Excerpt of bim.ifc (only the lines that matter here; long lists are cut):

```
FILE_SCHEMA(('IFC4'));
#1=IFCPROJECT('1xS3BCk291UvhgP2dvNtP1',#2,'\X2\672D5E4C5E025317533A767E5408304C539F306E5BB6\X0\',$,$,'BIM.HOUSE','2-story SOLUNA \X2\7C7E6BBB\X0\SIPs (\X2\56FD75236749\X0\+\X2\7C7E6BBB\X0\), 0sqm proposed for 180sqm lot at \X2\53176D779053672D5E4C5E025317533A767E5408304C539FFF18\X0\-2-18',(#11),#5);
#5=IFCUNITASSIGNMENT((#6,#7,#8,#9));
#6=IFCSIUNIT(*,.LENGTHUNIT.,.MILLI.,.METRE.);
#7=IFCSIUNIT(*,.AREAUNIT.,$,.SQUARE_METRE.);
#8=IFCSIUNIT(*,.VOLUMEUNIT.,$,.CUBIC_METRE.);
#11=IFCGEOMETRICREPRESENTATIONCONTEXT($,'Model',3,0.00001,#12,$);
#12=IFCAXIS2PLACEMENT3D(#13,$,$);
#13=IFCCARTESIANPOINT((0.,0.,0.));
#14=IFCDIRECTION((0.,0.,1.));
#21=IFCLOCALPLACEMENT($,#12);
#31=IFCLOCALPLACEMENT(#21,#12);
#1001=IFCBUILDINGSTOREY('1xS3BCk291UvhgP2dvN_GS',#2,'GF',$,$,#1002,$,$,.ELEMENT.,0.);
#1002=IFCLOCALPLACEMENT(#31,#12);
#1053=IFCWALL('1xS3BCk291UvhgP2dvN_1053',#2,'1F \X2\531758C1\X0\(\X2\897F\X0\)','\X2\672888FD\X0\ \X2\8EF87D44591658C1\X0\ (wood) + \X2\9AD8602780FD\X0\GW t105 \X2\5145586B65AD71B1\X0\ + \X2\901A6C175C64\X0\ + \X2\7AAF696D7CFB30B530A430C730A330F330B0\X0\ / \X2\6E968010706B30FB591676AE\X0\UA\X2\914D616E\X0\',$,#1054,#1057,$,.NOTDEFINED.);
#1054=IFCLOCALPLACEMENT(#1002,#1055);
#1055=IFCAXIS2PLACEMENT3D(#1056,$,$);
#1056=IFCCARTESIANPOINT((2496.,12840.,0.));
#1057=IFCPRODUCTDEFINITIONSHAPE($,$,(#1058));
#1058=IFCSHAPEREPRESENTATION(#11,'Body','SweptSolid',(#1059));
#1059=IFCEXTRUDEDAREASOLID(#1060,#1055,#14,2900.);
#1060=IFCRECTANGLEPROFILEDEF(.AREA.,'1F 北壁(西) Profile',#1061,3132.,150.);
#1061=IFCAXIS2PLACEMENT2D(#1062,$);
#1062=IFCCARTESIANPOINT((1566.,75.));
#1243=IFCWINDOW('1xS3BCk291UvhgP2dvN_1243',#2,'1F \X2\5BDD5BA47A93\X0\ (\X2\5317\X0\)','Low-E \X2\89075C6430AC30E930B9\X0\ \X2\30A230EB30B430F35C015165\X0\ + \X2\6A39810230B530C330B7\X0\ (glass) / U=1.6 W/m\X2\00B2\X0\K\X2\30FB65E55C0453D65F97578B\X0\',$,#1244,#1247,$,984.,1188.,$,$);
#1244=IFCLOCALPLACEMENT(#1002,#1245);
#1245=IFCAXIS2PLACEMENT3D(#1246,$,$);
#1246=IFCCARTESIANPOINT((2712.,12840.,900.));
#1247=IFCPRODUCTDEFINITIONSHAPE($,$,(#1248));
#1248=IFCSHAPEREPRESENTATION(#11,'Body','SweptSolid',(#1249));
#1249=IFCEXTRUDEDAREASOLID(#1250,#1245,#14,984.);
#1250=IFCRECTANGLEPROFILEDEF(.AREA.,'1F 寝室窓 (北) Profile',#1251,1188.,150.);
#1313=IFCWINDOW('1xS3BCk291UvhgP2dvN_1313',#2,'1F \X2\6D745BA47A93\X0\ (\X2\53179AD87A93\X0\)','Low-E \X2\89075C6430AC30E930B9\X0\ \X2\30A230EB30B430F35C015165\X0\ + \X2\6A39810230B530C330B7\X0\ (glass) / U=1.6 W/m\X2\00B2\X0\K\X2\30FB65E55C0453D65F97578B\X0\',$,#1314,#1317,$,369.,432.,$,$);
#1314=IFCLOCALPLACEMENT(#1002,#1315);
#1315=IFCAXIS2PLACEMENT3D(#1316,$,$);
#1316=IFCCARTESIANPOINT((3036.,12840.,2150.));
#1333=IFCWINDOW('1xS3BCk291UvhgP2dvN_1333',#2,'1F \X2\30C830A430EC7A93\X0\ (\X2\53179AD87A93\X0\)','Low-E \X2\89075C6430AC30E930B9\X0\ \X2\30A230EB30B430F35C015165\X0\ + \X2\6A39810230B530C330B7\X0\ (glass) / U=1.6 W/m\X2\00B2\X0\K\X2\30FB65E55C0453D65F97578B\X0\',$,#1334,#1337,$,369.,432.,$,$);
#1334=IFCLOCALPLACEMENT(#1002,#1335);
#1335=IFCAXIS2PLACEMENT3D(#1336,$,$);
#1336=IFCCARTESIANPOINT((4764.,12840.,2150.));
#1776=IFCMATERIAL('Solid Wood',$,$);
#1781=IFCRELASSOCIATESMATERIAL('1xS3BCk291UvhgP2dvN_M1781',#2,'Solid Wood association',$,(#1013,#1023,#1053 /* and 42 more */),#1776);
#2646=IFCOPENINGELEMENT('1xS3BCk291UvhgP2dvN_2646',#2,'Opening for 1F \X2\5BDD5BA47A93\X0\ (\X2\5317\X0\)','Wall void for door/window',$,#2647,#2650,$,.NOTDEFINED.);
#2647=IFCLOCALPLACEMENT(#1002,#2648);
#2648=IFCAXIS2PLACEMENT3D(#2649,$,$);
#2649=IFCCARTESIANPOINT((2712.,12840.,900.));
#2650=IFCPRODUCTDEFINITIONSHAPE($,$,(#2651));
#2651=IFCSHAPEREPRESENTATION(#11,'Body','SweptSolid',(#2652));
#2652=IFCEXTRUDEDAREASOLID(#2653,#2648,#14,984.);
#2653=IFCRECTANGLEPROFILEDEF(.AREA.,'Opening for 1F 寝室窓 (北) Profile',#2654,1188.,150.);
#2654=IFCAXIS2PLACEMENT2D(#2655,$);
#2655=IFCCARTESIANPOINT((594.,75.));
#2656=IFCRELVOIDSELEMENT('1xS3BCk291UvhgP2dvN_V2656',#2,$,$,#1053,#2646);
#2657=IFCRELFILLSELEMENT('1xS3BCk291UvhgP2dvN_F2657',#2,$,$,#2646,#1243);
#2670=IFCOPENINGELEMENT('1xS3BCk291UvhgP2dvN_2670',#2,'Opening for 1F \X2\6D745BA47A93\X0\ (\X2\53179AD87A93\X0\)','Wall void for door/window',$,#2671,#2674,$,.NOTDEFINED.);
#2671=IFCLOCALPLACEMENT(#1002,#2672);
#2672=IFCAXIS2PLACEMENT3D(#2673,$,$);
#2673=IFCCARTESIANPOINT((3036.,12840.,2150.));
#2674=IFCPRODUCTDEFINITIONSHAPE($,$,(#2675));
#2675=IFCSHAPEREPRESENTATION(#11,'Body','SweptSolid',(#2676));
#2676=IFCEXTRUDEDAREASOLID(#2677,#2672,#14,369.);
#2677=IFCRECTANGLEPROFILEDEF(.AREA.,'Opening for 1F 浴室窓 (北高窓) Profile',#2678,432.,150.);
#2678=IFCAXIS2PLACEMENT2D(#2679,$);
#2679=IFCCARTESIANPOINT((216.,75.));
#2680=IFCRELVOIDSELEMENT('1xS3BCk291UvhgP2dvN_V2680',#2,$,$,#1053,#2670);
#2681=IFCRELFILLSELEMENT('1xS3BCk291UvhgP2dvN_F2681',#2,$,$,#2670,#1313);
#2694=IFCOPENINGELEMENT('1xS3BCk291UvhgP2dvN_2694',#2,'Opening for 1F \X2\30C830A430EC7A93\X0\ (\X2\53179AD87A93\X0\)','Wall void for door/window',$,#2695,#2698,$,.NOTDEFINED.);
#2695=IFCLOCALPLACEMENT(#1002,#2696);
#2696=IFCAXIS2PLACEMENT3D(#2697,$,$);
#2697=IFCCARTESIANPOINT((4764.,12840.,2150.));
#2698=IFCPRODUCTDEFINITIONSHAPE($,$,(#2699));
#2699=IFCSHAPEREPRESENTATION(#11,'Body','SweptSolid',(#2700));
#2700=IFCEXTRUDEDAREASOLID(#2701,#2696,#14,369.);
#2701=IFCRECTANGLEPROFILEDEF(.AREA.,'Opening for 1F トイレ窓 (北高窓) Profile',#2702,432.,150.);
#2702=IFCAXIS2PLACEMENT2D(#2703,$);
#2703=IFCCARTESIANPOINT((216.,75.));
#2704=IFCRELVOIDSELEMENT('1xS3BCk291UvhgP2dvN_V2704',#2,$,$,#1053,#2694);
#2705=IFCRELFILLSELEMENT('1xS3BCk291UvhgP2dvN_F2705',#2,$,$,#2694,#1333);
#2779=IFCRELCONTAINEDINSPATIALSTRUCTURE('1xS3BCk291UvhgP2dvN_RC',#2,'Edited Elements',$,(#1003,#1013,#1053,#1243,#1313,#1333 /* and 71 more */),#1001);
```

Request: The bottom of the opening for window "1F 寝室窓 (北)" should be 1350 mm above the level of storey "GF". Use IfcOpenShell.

```python
import numpy as np
import ifcopenshell
import ifcopenshell.api.geometry
import ifcopenshell.geom
import ifcopenshell.util.element
import ifcopenshell.util.placement
import ifcopenshell.util.shape
import ifcopenshell.util.unit

model = ifcopenshell.open("bim.ifc")
unit_scale = ifcopenshell.util.unit.calculate_unit_scale(model)

window = model.by_guid("1xS3BCk291UvhgP2dvN_1243")
opening = window.FillsVoids[0].RelatingOpeningElement
storey = ifcopenshell.util.element.get_container(window, ifc_class="IfcBuildingStorey")
level = ifcopenshell.util.placement.get_local_placement(storey.ObjectPlacement)[2, 3]

# The opening's origin need not be at the sill, so measure its lowest point.
shape = ifcopenshell.geom.create_shape(ifcopenshell.geom.settings(), opening)
bottom = ifcopenshell.util.shape.get_shape_bottom_elevation(shape, shape.geometry) / unit_scale
dz = level + 1.35 / unit_scale - bottom

shift = np.array([0.0, 0.0, dz])
# The window is not placed relative to its opening, so move both.
for product in (opening, window):
    matrix = ifcopenshell.util.placement.get_local_placement(product.ObjectPlacement)
    matrix[:3, 3] += shift
    ifcopenshell.api.geometry.edit_object_placement(model, product=product, matrix=matrix, is_si=False)

print(f"moved by {dz * unit_scale:+.3f} m")

model.write("bim_updated.ifc")
```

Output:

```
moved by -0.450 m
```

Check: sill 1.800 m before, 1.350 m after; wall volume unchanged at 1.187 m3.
